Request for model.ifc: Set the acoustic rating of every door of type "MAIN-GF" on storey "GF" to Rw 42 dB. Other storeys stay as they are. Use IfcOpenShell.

First a look at what the model holds.

```python
import ifcopenshell
import ifcopenshell.util.element

model = ifcopenshell.open("model.ifc")
print(model.schema)
storey = next(s for s in model.by_type("IfcBuildingStorey") if s.Name == "GF")
doors = [e for e in ifcopenshell.util.element.get_decomposition(storey) if e.is_a("IfcDoor")]
seen = {}
for e in doors:
    element_type = ifcopenshell.util.element.get_type(e)
    key = (element_type.Name if element_type != e and element_type else None, ifcopenshell.util.element.get_pset(e, "Pset_DoorCommon", "AcousticRating"))
    seen[key] = seen.get(key, 0) + 1
for (name, value), count in sorted(seen.items(), key=str):
    print(count, "x", name, "|", value)
```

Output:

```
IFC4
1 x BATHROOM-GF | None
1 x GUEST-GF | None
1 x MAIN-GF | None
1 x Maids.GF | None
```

```python
import ifcopenshell
import ifcopenshell.api.pset
import ifcopenshell.util.element

model = ifcopenshell.open("model.ifc")

storey = next(s for s in model.by_type("IfcBuildingStorey") if s.Name == "GF")
doors = [e for e in ifcopenshell.util.element.get_decomposition(storey) if e.is_a("IfcDoor")]

count = 0
for e in doors:
    element_type = ifcopenshell.util.element.get_type(e)
    if element_type in (None, e) or element_type.Name != "MAIN-GF":
        continue
    # add_pset returns the element's existing set when there is one.
    pset = ifcopenshell.api.pset.add_pset(model, product=e, name="Pset_DoorCommon")
    ifcopenshell.api.pset.edit_pset(model, pset=pset, properties={"AcousticRating": "Rw 42 dB"})
    count += 1

print(count, "doors updated")

model.write("model_updated.ifc")
```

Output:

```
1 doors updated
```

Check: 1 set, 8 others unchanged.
